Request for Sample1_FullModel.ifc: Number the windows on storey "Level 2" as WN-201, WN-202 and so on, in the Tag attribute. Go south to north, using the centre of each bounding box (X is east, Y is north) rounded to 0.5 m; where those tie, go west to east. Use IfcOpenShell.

First a look at what the model holds.

```python
import ifcopenshell
import ifcopenshell.util.element
import ifcopenshell.util.placement

model = ifcopenshell.open("Sample1_FullModel.ifc")
print(model.schema)
storey = next(s for s in model.by_type("IfcBuildingStorey") if s.Name == "Level 2")
windows = [e for e in ifcopenshell.util.element.get_decomposition(storey) if e.is_a("IfcWindow")]
for e in sorted(windows, key=lambda e: e.id()):
    origin = ifcopenshell.util.placement.get_local_placement(e.ObjectPlacement)[:3, 3]
    print(e.id(), e.Tag, e.Name, origin.round(2) + 0.0, sep=" | ")
```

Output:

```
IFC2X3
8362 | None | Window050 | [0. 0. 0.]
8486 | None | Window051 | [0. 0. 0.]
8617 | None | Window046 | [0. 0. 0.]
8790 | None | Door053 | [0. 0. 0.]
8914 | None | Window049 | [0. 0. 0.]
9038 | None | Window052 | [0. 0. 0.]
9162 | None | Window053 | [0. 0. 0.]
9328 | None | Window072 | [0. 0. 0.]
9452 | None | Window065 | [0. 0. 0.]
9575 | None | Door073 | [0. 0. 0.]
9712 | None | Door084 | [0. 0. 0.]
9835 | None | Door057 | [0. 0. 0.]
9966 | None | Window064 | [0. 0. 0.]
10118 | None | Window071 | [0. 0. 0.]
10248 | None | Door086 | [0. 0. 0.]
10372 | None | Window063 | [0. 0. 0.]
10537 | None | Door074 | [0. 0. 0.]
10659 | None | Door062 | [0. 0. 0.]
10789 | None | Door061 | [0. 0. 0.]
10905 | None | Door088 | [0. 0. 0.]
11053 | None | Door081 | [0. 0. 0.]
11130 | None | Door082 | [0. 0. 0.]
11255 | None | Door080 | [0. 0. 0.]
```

```python
import ifcopenshell
import ifcopenshell.geom
import ifcopenshell.util.element
import ifcopenshell.util.shape

model = ifcopenshell.open("Sample1_FullModel.ifc")
settings = ifcopenshell.geom.settings()
settings.set("use-world-coords", True)


def centre(element):
    shape = ifcopenshell.geom.create_shape(settings, element)
    return ifcopenshell.util.shape.get_bbox_centroid(shape.geometry)


storey = next(s for s in model.by_type("IfcBuildingStorey") if s.Name == "Level 2")
windows = [e for e in ifcopenshell.util.element.get_decomposition(storey) if e.is_a("IfcWindow")]

# Insertion points can sit at a corner or the storey origin, so sort by the geometry (in metres).
centres = {e: centre(e) for e in windows}
windows.sort(key=lambda e: (round(centres[e][1] / 0.5), centres[e][0]))

for i, e in enumerate(windows, start=1):
    number = f"WN-2{i:02d}"
    e.Tag = number
    print(e.id(), number)

model.write("Sample1_FullModel_updated.ifc")
```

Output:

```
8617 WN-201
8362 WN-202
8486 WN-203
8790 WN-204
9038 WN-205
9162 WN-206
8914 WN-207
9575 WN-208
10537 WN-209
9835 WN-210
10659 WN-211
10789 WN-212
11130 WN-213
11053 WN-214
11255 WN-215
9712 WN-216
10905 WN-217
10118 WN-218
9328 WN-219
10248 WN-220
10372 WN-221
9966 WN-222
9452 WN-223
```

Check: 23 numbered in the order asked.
